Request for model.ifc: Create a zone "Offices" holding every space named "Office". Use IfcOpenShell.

First a look at what the model holds.

```python
import ifcopenshell

model = ifcopenshell.open("model.ifc")
print(model.schema)
seen = {}
for space in model.by_type("IfcSpace"):
    seen[space.LongName] = seen.get(space.LongName, 0) + 1
for name, count in sorted(seen.items(), key=str):
    print(count, "x", name)
print("zones:", [z.Name for z in model.by_type("IfcZone")][:20])
```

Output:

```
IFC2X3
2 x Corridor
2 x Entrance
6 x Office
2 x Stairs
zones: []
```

```python
import ifcopenshell
import ifcopenshell.api.group
import ifcopenshell.api.root

model = ifcopenshell.open("model.ifc")

names = {"Office"}
spaces = [s for s in model.by_type("IfcSpace") if s.LongName in names]

zone = ifcopenshell.api.root.create_entity(model, ifc_class="IfcZone", name="Offices")
ifcopenshell.api.group.assign_group(model, products=spaces, group=zone)
print(len(spaces), "spaces in", zone.Name)

model.write("model_v2.ifc")
```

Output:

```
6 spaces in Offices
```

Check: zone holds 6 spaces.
